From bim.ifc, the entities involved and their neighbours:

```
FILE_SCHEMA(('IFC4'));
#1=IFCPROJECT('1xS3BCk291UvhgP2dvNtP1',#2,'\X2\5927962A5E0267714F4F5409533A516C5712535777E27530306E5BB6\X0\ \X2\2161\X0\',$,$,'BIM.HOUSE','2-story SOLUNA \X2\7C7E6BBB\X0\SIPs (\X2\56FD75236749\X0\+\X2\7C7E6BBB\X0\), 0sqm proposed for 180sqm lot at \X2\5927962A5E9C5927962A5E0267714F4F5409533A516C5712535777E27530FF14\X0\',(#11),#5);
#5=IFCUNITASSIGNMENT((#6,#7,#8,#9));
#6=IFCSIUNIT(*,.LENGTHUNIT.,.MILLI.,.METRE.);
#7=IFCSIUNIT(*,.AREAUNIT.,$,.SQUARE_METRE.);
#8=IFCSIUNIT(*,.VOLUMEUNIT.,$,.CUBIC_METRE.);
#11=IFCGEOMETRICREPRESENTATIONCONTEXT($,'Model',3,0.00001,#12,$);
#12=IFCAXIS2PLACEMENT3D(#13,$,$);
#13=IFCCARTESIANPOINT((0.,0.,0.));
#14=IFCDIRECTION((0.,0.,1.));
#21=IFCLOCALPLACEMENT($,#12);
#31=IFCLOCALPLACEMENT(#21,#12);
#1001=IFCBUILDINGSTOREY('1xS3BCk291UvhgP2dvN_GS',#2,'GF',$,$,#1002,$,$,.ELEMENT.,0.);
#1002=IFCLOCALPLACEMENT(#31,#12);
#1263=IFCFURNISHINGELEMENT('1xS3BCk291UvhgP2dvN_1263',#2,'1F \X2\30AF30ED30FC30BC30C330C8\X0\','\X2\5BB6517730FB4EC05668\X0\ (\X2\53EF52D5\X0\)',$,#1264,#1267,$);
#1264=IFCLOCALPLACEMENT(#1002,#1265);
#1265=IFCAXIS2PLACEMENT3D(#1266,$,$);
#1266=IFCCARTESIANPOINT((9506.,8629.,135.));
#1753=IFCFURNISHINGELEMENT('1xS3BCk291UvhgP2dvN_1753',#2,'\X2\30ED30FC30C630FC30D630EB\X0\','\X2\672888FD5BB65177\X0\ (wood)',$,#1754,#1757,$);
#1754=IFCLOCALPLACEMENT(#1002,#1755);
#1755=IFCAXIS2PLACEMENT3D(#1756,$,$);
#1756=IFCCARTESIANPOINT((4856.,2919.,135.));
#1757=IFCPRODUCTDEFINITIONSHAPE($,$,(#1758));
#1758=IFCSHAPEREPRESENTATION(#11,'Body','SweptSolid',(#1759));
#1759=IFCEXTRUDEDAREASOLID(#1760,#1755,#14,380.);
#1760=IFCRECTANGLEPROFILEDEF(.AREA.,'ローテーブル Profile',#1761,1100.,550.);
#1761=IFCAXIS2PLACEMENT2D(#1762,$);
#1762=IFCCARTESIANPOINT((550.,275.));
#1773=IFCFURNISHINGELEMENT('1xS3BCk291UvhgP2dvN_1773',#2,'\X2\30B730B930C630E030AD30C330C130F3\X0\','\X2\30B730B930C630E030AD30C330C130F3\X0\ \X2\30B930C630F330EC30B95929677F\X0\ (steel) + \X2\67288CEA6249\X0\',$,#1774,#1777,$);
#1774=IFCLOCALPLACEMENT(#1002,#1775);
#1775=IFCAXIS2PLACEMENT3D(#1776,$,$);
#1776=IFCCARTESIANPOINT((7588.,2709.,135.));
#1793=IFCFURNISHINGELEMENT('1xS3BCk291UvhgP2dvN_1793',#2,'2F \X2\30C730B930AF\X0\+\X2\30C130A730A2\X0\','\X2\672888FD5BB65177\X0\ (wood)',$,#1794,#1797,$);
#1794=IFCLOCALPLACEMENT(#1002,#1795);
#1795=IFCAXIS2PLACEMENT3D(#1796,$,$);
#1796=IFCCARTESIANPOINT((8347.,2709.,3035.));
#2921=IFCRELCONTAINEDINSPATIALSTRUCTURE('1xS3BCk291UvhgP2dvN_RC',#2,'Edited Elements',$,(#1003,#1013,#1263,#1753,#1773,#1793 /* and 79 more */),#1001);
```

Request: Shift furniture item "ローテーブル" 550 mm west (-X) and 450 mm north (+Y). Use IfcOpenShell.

```python
import ifcopenshell
import ifcopenshell.api.geometry
import ifcopenshell.util.placement

model = ifcopenshell.open("bim.ifc")

item = model.by_guid("1xS3BCk291UvhgP2dvN_1753")
matrix = ifcopenshell.util.placement.get_local_placement(item.ObjectPlacement)
matrix[0, 3] -= 550.0
matrix[1, 3] += 450.0
ifcopenshell.api.geometry.edit_object_placement(model, product=item, matrix=matrix, is_si=False)

print(ifcopenshell.util.placement.get_local_placement(item.ObjectPlacement).round(3) + 0.0)

model.write("bim_v2.ifc")
```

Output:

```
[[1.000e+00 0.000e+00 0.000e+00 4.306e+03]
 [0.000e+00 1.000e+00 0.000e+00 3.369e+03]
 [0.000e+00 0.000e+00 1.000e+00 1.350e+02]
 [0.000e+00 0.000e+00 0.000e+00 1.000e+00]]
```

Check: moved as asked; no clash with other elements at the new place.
